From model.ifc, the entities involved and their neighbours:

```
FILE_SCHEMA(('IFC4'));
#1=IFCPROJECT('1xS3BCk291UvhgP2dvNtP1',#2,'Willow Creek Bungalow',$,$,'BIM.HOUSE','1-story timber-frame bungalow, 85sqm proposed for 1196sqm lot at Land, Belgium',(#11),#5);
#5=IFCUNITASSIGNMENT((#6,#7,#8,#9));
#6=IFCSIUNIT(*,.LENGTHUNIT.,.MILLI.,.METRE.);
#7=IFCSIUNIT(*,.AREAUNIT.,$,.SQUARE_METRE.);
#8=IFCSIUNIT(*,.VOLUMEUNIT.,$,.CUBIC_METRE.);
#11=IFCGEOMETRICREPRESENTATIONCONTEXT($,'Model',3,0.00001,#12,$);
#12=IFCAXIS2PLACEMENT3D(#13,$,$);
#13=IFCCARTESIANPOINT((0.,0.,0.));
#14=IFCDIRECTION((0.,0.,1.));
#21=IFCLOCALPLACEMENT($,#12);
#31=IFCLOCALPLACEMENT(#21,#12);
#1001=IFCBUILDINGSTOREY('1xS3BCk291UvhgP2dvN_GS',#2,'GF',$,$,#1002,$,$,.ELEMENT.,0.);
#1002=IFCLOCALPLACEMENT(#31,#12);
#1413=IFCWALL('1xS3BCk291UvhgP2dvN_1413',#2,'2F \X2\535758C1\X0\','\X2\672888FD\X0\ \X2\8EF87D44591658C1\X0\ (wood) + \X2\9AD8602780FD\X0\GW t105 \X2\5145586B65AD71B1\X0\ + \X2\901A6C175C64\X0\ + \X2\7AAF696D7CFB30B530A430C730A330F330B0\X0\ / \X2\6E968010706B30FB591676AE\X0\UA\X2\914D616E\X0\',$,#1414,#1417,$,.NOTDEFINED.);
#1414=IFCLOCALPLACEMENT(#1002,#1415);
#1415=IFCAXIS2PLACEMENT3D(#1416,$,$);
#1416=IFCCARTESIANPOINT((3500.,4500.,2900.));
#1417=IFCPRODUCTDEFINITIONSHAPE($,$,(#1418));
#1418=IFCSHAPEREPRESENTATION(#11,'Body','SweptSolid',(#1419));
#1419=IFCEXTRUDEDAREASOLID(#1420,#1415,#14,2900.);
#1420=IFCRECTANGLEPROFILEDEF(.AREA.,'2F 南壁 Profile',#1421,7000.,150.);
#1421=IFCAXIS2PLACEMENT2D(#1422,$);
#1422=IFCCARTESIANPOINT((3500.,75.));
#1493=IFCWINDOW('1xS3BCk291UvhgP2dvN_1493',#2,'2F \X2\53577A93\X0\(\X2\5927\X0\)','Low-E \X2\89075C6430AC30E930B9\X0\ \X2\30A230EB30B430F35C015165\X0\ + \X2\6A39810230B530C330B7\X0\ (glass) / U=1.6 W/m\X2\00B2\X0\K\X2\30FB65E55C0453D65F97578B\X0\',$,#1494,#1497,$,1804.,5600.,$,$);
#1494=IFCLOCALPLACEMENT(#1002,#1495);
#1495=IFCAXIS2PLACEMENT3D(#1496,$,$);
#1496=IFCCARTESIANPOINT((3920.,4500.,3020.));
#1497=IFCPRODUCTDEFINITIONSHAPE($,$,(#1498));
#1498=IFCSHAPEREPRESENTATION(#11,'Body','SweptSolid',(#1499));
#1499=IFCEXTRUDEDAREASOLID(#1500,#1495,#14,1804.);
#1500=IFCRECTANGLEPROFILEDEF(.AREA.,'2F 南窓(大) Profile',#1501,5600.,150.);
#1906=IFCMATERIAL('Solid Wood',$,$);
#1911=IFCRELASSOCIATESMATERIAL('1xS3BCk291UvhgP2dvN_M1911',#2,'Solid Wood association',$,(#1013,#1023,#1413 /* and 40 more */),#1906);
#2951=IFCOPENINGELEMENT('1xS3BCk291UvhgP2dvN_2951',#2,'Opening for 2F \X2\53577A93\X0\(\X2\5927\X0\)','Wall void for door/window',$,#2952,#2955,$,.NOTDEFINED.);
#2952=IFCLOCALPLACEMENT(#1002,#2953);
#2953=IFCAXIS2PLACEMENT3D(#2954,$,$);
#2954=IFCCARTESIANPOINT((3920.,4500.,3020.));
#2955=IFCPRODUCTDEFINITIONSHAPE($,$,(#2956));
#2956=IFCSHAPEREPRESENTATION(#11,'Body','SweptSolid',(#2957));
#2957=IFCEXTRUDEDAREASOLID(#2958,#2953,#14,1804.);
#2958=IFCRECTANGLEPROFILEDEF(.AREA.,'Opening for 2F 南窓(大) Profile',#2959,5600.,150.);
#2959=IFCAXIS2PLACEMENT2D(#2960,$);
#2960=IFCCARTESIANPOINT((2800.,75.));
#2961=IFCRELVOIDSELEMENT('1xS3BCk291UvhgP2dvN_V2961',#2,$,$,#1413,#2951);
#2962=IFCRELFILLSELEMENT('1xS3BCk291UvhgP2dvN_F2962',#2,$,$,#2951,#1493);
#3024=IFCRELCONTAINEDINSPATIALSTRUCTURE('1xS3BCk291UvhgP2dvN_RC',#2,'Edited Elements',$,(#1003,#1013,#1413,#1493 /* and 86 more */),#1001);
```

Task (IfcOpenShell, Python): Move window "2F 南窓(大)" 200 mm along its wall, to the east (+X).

```python
import ifcopenshell
import ifcopenshell.api.geometry
import ifcopenshell.util.placement

model = ifcopenshell.open("model.ifc")

window = model.by_id(1493)
opening = window.FillsVoids[0].RelatingOpeningElement
wall = opening.VoidsElements[0].RelatingBuildingElement

wall_matrix = ifcopenshell.util.placement.get_local_placement(wall.ObjectPlacement)
shift = wall_matrix[:3, 0] * 200.0
before = ifcopenshell.util.placement.get_local_placement(window.ObjectPlacement)[:3, 3].copy()

# The window is not placed relative to its opening, so move both.
for product in (opening, window):
    matrix = ifcopenshell.util.placement.get_local_placement(product.ObjectPlacement)
    matrix[:3, 3] += shift
    ifcopenshell.api.geometry.edit_object_placement(model, product=product, matrix=matrix, is_si=False)

after = ifcopenshell.util.placement.get_local_placement(window.ObjectPlacement)[:3, 3]
print("window moved by", (after - before).round(3) + 0.0)

model.write("model_v2.ifc")
```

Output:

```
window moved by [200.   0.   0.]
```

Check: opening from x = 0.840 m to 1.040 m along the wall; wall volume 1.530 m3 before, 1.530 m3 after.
